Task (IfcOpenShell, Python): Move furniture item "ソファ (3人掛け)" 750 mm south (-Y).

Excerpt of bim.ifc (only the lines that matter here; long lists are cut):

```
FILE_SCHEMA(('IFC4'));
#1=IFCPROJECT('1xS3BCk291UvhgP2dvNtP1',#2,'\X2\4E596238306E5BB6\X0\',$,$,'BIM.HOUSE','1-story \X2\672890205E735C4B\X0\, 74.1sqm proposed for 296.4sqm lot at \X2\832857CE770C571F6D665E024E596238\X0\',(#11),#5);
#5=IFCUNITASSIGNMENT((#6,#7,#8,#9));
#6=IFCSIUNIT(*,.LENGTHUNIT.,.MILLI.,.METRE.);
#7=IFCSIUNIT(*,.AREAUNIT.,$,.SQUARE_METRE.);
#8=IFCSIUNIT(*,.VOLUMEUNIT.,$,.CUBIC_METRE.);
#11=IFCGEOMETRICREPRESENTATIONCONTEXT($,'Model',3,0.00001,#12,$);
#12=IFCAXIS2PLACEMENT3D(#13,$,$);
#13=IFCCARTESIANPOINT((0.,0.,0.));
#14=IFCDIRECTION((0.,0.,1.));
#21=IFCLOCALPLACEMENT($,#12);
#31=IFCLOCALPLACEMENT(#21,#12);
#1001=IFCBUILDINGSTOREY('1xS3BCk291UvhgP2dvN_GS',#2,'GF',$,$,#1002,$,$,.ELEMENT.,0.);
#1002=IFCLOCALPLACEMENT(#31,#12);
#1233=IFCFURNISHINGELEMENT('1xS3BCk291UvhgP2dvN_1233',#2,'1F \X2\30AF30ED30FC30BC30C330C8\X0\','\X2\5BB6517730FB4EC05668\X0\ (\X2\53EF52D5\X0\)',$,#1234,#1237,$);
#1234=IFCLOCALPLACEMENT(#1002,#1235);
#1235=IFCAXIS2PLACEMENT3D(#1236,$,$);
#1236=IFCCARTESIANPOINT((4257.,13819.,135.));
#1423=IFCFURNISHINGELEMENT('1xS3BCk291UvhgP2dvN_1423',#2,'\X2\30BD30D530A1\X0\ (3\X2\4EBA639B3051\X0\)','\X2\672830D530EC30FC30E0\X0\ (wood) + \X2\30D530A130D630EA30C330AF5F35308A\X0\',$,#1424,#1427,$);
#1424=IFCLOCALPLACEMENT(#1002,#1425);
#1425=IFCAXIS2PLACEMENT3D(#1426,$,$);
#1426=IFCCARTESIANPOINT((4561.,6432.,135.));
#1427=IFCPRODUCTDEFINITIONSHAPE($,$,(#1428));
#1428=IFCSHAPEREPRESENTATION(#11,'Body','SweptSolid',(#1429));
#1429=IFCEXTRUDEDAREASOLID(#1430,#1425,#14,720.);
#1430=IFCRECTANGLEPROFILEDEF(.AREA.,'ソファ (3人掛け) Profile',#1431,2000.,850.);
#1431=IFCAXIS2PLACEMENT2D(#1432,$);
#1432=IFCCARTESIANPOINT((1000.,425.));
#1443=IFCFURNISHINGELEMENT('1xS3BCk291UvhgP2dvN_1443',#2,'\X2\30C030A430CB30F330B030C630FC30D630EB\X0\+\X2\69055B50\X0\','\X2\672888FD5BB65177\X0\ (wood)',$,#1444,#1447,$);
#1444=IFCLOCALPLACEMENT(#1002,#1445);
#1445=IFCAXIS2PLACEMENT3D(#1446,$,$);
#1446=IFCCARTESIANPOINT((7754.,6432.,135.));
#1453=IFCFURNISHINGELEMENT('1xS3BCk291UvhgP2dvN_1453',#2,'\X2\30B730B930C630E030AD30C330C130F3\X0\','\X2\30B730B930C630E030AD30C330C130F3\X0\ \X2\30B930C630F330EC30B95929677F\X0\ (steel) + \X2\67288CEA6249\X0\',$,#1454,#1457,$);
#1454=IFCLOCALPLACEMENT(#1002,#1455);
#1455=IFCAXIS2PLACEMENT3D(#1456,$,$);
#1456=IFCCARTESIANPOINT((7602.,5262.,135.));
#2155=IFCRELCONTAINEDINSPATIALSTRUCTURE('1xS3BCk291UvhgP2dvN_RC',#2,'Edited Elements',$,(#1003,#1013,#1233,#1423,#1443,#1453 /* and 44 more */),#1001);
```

```python
import ifcopenshell
import ifcopenshell.api.geometry
import ifcopenshell.util.placement

model = ifcopenshell.open("bim.ifc")

item = model.by_id(1423)
matrix = ifcopenshell.util.placement.get_local_placement(item.ObjectPlacement)
matrix[1, 3] -= 750.0
ifcopenshell.api.geometry.edit_object_placement(model, product=item, matrix=matrix, is_si=False)

print(ifcopenshell.util.placement.get_local_placement(item.ObjectPlacement).round(3) + 0.0)

model.write("bim-out.ifc")
```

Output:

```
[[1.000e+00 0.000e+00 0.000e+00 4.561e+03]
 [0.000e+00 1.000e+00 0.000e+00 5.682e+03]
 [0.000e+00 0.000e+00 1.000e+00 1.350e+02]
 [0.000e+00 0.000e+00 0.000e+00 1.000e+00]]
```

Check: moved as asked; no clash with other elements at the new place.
